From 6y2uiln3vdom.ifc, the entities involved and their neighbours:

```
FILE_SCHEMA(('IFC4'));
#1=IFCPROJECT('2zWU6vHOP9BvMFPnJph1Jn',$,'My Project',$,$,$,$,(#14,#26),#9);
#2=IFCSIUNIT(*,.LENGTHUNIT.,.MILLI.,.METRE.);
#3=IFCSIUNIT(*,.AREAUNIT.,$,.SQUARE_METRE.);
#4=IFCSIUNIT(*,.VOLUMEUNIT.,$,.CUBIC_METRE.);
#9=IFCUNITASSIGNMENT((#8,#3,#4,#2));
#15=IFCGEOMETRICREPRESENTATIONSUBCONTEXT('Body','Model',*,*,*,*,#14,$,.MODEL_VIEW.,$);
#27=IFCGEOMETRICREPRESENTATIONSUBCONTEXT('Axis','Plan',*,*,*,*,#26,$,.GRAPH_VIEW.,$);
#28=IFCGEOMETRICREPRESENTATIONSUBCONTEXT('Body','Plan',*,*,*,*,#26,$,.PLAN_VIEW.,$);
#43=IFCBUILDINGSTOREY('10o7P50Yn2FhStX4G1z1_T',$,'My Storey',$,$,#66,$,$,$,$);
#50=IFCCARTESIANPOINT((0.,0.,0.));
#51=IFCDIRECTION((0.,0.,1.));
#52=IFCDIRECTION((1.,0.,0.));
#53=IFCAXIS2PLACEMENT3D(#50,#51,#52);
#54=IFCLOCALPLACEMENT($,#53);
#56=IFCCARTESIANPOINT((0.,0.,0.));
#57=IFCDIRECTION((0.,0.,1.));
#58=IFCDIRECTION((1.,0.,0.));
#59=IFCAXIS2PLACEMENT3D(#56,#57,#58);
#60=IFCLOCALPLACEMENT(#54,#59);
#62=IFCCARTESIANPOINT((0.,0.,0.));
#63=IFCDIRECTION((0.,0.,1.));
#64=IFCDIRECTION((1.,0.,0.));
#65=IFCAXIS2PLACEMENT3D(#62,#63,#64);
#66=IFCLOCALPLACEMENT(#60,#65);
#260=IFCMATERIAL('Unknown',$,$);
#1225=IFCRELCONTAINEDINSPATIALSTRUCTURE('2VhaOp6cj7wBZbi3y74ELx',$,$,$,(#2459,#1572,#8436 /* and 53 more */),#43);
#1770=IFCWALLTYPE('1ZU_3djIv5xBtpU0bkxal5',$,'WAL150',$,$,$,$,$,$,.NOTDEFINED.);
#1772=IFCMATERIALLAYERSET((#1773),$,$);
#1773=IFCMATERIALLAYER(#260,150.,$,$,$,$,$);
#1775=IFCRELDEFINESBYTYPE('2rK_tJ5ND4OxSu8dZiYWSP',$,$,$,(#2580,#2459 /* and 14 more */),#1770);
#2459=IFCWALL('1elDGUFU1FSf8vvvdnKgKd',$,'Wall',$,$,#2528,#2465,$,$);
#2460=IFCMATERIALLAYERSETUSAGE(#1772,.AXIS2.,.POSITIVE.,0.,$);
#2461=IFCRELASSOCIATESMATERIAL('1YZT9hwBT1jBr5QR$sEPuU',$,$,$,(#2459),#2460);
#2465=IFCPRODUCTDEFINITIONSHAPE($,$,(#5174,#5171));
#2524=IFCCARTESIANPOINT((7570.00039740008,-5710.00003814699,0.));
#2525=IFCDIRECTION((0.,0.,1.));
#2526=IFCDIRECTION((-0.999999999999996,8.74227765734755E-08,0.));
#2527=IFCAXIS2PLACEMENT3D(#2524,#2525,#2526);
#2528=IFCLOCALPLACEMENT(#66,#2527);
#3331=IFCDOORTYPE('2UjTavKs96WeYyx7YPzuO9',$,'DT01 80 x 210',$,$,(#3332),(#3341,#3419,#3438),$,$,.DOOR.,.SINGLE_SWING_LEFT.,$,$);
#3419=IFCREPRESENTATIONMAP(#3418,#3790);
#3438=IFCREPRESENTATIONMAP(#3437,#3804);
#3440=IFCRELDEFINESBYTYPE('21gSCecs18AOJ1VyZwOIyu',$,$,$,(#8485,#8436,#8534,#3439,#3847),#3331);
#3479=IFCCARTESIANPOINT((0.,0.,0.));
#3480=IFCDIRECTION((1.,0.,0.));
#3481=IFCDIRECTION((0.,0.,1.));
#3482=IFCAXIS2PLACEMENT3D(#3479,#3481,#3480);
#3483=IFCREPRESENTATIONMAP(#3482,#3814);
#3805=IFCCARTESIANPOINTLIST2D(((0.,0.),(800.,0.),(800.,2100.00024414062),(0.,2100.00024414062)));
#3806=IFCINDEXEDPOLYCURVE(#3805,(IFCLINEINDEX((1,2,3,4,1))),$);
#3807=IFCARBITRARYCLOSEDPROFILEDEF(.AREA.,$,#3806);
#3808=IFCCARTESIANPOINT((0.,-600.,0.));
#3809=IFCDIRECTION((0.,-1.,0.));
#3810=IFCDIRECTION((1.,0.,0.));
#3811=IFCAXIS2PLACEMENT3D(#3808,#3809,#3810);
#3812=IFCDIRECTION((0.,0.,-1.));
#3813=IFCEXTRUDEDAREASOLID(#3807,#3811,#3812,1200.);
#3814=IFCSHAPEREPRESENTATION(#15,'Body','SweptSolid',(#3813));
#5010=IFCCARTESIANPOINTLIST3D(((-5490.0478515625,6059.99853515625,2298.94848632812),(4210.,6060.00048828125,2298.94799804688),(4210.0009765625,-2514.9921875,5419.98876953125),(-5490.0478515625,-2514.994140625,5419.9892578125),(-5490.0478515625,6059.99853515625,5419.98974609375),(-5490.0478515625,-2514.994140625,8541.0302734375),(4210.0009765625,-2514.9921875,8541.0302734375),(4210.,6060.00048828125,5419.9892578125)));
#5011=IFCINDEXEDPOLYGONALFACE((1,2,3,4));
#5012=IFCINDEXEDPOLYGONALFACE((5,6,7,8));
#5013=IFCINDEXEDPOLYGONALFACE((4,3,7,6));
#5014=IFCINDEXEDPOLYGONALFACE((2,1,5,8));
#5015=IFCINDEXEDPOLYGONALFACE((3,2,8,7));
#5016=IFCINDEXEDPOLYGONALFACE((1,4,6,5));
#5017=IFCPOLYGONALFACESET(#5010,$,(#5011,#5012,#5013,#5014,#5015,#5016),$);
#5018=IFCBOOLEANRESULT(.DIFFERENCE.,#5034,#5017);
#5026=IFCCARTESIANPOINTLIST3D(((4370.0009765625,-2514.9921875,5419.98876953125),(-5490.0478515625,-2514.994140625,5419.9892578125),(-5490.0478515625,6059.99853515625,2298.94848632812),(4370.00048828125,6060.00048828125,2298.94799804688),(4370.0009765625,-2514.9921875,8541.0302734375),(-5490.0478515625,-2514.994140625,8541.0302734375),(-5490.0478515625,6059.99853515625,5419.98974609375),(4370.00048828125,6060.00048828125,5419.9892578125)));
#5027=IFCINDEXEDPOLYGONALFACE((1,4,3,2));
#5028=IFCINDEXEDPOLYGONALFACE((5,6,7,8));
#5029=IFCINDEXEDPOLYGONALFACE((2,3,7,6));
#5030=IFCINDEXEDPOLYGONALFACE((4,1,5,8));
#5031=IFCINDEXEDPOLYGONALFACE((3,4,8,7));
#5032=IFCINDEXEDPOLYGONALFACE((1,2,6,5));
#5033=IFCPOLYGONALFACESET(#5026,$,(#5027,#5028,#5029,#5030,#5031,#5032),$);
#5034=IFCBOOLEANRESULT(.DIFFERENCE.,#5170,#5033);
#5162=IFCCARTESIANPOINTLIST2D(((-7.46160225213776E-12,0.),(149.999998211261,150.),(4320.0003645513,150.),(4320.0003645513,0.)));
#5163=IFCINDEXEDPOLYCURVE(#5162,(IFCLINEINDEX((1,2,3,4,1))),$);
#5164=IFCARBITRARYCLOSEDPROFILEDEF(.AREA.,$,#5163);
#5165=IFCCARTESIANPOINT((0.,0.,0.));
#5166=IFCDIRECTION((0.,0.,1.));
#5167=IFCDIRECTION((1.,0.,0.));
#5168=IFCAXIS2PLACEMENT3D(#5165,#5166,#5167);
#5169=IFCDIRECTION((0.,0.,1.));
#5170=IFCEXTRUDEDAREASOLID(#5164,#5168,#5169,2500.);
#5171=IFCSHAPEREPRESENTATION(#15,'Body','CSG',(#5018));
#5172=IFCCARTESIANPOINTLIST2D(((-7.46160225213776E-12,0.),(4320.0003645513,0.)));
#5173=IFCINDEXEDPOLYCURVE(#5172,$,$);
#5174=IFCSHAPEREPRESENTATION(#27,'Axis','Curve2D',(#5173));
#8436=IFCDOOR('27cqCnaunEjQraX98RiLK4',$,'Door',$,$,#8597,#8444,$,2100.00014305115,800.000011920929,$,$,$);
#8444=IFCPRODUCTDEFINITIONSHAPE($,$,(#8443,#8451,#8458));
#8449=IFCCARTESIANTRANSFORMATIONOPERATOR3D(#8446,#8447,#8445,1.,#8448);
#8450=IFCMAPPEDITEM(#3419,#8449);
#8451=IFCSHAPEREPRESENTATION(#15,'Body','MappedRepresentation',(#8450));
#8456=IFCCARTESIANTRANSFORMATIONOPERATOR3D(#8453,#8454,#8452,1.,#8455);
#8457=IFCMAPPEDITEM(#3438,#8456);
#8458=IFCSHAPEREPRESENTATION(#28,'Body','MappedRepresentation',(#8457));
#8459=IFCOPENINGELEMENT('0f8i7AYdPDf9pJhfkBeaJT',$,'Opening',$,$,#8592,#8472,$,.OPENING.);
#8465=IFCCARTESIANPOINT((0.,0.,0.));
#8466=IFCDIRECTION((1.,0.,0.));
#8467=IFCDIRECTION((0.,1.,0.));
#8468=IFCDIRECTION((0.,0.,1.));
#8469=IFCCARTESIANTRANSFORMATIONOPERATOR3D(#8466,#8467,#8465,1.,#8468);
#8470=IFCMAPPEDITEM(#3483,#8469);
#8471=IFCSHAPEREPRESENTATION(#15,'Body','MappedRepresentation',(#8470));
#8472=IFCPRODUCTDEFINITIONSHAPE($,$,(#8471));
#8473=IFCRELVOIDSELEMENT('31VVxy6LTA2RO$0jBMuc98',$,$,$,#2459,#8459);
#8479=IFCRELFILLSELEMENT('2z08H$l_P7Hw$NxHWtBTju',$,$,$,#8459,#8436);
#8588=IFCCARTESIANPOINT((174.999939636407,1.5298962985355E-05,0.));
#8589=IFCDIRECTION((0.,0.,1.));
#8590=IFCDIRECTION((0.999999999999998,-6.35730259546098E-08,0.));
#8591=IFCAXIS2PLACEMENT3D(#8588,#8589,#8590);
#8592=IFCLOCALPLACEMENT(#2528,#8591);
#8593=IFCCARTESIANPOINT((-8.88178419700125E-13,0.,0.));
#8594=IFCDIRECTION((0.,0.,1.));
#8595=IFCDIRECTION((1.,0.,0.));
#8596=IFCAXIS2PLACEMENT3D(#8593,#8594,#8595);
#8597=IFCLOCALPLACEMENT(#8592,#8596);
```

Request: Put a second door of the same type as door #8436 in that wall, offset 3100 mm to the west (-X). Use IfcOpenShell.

```python
import ifcopenshell
import ifcopenshell.api.feature
import ifcopenshell.api.geometry
import ifcopenshell.api.root
import ifcopenshell.geom
import ifcopenshell.util.element
import ifcopenshell.util.placement
import ifcopenshell.util.shape
import ifcopenshell.util.unit

model = ifcopenshell.open("6y2uiln3vdom.ifc")
unit_scale = ifcopenshell.util.unit.calculate_unit_scale(model)
settings = ifcopenshell.geom.settings()


def volume(element):
    """Net volume in cubic metres, openings subtracted."""
    shape = ifcopenshell.geom.create_shape(settings, element)
    return ifcopenshell.util.shape.get_volume(shape.geometry)


door = model.by_guid("27cqCnaunEjQraX98RiLK4")
opening = door.FillsVoids[0].RelatingOpeningElement
wall = opening.VoidsElements[0].RelatingBuildingElement
before = volume(wall)
shift = ifcopenshell.util.placement.get_local_placement(wall.ObjectPlacement)[:3, 0] * 3.1 / unit_scale

# copy_class copies the void relationship, type, container and properties, but no geometry.
new_opening = ifcopenshell.api.root.copy_class(model, product=opening)
new_opening.Representation = ifcopenshell.util.element.copy_deep(
    model, opening.Representation, exclude=["IfcGeometricRepresentationContext", "IfcRepresentationMap"]
)
new_door = ifcopenshell.api.root.copy_class(model, product=door)
new_door.Representation = ifcopenshell.util.element.copy_deep(
    model, door.Representation, exclude=["IfcGeometricRepresentationContext", "IfcRepresentationMap"]
)
ifcopenshell.api.feature.add_filling(model, opening=new_opening, element=new_door)

for old, new in ((opening, new_opening), (door, new_door)):
    matrix = ifcopenshell.util.placement.get_local_placement(old.ObjectPlacement)
    matrix[:3, 3] += shift
    ifcopenshell.api.geometry.edit_object_placement(model, product=new, matrix=matrix, is_si=False)

after = volume(wall)

print(f"wall volume {before:.3f} -> {after:.3f} m3")

model.write("6y2uiln3vdom_rev.ifc")
```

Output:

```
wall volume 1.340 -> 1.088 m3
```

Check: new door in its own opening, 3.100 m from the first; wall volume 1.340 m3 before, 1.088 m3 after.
